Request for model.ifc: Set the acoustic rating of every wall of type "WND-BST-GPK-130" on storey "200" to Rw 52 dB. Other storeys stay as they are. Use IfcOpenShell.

First a look at what the model holds.

```python
import ifcopenshell
import ifcopenshell.util.element

model = ifcopenshell.open("model.ifc")
print(model.schema)
storey = next(s for s in model.by_type("IfcBuildingStorey") if s.Name == "200")
walls = [e for e in ifcopenshell.util.element.get_decomposition(storey) if e.is_a("IfcWall")]
seen = {}
for e in walls:
    element_type = ifcopenshell.util.element.get_type(e)
    key = (element_type.Name if element_type != e and element_type else None, ifcopenshell.util.element.get_pset(e, "Pset_WallCommon", "AcousticRating"))
    seen[key] = seen.get(key, 0) + 1
for (name, value), count in sorted(seen.items(), key=str):
    print(count, "x", name, "|", value)
```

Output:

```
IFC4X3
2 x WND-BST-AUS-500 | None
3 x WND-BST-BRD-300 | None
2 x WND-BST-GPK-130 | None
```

```python
import ifcopenshell
import ifcopenshell.api.pset
import ifcopenshell.util.element

model = ifcopenshell.open("model.ifc")

storey = next(s for s in model.by_type("IfcBuildingStorey") if s.Name == "200")
walls = [e for e in ifcopenshell.util.element.get_decomposition(storey) if e.is_a("IfcWall")]

count = 0
for e in walls:
    element_type = ifcopenshell.util.element.get_type(e)
    if element_type in (None, e) or element_type.Name != "WND-BST-GPK-130":
        continue
    # add_pset returns the element's existing set when there is one.
    pset = ifcopenshell.api.pset.add_pset(model, product=e, name="Pset_WallCommon")
    ifcopenshell.api.pset.edit_pset(model, pset=pset, properties={"AcousticRating": "Rw 52 dB"})
    count += 1

print(count, "walls updated")

model.write("model-out.ifc")
```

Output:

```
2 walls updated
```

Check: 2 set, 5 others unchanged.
